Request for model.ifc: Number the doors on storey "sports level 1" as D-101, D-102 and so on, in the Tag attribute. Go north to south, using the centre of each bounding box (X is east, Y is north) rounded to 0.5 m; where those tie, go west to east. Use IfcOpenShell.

First a look at what the model holds.

```python
import ifcopenshell
import ifcopenshell.util.element
import ifcopenshell.util.placement

model = ifcopenshell.open("model.ifc")
print(model.schema)
storey = next(s for s in model.by_type("IfcBuildingStorey") if s.Name == "sports level 1")
doors = [e for e in ifcopenshell.util.element.get_decomposition(storey) if e.is_a("IfcDoor")]
for e in sorted(doors, key=lambda e: e.id()):
    origin = ifcopenshell.util.placement.get_local_placement(e.ObjectPlacement)[:3, 3]
    print(e.id(), e.Tag, e.Name, origin.round(2) + 0.0, sep=" | ")
```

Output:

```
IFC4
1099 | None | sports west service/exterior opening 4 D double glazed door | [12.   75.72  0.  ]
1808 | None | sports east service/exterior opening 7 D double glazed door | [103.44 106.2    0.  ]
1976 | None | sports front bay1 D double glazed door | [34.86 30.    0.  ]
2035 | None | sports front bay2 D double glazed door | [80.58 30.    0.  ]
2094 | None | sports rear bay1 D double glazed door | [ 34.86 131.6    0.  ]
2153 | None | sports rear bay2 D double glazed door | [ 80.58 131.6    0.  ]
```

```python
import ifcopenshell
import ifcopenshell.geom
import ifcopenshell.util.element
import ifcopenshell.util.shape

model = ifcopenshell.open("model.ifc")
settings = ifcopenshell.geom.settings()
settings.set("use-world-coords", True)


def centre(element):
    shape = ifcopenshell.geom.create_shape(settings, element)
    return ifcopenshell.util.shape.get_bbox_centroid(shape.geometry)


storey = next(s for s in model.by_type("IfcBuildingStorey") if s.Name == "sports level 1")
doors = [e for e in ifcopenshell.util.element.get_decomposition(storey) if e.is_a("IfcDoor")]

# Insertion points can sit at a corner or the storey origin, so sort by the geometry (in metres).
centres = {e: centre(e) for e in doors}
doors.sort(key=lambda e: (-round(centres[e][1] / 0.5), centres[e][0]))

for i, e in enumerate(doors, start=1):
    number = f"D-1{i:02d}"
    e.Tag = number
    print(e.id(), number)

model.write("model_rev.ifc")
```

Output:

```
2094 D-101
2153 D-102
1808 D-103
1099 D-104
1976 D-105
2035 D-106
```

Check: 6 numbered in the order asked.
